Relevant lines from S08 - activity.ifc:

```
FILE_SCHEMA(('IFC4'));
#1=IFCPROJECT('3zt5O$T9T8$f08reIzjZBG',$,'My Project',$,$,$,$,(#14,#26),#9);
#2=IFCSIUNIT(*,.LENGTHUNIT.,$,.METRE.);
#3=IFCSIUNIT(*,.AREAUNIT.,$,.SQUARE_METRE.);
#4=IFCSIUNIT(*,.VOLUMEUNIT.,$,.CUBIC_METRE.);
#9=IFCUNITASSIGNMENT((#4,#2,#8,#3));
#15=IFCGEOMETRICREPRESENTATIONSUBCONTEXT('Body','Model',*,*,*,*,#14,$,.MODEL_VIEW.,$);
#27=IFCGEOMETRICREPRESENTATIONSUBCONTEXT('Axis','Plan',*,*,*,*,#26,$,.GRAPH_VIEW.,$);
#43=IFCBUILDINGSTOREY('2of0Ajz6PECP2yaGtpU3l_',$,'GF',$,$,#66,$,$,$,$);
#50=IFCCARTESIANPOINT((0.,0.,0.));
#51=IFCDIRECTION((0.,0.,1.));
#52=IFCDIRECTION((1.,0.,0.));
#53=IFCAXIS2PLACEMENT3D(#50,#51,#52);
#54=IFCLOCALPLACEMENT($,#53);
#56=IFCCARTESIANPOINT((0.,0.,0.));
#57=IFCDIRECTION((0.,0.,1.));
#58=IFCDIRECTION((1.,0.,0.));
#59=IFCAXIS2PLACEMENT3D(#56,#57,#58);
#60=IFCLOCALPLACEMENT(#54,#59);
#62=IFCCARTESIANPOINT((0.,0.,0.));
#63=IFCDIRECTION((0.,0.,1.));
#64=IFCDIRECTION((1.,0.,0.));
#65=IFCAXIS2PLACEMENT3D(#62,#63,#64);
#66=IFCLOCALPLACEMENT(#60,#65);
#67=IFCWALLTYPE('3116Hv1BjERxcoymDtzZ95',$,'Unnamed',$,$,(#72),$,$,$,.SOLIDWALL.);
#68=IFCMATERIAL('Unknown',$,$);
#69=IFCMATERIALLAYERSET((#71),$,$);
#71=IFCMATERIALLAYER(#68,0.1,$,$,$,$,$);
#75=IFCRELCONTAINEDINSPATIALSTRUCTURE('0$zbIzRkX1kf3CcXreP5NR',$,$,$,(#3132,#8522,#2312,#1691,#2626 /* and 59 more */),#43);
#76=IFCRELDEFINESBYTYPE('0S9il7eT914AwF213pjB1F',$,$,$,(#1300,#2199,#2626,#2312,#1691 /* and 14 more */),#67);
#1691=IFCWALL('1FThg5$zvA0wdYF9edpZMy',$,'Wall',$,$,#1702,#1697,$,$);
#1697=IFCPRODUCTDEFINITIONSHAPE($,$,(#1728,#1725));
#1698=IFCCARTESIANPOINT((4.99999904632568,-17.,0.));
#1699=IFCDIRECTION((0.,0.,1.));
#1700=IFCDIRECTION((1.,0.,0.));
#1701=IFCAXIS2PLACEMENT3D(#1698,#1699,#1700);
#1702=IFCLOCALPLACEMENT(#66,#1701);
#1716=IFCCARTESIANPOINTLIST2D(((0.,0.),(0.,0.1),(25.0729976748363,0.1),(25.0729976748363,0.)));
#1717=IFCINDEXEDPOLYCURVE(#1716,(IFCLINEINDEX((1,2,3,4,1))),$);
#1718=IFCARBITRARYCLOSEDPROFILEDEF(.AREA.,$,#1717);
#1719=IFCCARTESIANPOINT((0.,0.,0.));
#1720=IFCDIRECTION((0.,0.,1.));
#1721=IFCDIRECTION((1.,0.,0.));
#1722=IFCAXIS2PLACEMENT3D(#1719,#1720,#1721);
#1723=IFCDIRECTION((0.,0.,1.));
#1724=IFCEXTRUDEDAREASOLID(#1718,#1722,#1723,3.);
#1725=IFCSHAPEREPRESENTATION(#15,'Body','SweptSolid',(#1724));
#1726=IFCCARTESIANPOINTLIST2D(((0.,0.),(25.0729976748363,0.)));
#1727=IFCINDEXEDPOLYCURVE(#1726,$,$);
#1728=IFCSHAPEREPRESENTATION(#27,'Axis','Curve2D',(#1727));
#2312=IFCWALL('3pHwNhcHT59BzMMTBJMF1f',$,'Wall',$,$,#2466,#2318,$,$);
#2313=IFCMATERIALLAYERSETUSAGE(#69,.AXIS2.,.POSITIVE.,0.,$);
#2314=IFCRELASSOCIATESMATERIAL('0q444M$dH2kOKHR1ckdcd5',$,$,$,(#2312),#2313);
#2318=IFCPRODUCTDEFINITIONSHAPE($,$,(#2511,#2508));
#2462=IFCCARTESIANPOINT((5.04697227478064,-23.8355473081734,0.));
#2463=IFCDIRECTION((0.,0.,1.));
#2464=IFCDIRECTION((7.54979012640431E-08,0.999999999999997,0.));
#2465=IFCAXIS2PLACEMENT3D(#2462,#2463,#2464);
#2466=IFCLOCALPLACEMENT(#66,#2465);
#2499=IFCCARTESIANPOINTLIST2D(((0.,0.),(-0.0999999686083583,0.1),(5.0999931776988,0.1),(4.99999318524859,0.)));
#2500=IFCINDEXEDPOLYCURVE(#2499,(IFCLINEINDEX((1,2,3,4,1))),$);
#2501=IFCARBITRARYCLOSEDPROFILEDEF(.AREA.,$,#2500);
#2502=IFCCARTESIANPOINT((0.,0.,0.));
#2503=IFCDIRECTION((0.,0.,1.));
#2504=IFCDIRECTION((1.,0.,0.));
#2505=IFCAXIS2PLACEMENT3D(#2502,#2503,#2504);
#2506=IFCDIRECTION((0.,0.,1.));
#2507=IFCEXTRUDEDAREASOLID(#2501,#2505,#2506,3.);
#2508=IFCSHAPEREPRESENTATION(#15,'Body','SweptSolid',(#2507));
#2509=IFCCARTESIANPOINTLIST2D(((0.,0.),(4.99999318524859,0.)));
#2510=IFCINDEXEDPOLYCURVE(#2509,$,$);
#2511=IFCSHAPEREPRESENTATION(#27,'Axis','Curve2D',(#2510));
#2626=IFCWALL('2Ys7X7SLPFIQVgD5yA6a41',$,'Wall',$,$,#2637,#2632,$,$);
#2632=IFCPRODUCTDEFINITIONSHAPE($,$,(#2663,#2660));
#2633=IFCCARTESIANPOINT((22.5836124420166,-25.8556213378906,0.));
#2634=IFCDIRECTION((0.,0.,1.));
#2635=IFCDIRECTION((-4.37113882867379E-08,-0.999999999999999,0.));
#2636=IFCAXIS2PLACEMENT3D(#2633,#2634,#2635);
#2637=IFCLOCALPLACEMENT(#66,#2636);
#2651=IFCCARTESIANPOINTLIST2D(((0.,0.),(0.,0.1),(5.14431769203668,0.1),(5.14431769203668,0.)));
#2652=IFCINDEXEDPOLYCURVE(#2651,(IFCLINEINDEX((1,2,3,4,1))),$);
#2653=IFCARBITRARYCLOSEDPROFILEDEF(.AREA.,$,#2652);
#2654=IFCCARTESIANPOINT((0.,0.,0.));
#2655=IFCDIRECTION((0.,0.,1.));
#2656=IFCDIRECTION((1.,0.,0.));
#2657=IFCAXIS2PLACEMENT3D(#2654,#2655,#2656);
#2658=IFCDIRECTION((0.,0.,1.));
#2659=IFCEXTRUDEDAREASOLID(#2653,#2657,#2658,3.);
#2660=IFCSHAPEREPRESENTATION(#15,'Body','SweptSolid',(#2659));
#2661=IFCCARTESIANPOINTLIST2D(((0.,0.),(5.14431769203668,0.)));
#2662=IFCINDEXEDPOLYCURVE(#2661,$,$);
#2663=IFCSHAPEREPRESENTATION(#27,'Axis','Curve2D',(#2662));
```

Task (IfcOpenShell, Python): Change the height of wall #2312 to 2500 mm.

```python
import ifcopenshell
import ifcopenshell.geom
import ifcopenshell.util.representation
import ifcopenshell.util.shape

model = ifcopenshell.open("S08 - activity.ifc")
settings = ifcopenshell.geom.settings()


def volume(element):
    """Net volume in cubic metres, openings subtracted."""
    shape = ifcopenshell.geom.create_shape(settings, element)
    return ifcopenshell.util.shape.get_volume(shape.geometry)


wall = model.by_guid("3pHwNhcHT59BzMMTBJMF1f")
before = volume(wall)

body = ifcopenshell.util.representation.get_representation(wall, "Model", "Body")
solid = body.Items[0]
old_height = solid.Depth
solid.Depth = 2.5
after = volume(wall)

print(f"height {old_height:g} -> {solid.Depth:g}, volume {before:.3f} -> {after:.3f} m3")

model.write("S08 - activity_updated.ifc")
```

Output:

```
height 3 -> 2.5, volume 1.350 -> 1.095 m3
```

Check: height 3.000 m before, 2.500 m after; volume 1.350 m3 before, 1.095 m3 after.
